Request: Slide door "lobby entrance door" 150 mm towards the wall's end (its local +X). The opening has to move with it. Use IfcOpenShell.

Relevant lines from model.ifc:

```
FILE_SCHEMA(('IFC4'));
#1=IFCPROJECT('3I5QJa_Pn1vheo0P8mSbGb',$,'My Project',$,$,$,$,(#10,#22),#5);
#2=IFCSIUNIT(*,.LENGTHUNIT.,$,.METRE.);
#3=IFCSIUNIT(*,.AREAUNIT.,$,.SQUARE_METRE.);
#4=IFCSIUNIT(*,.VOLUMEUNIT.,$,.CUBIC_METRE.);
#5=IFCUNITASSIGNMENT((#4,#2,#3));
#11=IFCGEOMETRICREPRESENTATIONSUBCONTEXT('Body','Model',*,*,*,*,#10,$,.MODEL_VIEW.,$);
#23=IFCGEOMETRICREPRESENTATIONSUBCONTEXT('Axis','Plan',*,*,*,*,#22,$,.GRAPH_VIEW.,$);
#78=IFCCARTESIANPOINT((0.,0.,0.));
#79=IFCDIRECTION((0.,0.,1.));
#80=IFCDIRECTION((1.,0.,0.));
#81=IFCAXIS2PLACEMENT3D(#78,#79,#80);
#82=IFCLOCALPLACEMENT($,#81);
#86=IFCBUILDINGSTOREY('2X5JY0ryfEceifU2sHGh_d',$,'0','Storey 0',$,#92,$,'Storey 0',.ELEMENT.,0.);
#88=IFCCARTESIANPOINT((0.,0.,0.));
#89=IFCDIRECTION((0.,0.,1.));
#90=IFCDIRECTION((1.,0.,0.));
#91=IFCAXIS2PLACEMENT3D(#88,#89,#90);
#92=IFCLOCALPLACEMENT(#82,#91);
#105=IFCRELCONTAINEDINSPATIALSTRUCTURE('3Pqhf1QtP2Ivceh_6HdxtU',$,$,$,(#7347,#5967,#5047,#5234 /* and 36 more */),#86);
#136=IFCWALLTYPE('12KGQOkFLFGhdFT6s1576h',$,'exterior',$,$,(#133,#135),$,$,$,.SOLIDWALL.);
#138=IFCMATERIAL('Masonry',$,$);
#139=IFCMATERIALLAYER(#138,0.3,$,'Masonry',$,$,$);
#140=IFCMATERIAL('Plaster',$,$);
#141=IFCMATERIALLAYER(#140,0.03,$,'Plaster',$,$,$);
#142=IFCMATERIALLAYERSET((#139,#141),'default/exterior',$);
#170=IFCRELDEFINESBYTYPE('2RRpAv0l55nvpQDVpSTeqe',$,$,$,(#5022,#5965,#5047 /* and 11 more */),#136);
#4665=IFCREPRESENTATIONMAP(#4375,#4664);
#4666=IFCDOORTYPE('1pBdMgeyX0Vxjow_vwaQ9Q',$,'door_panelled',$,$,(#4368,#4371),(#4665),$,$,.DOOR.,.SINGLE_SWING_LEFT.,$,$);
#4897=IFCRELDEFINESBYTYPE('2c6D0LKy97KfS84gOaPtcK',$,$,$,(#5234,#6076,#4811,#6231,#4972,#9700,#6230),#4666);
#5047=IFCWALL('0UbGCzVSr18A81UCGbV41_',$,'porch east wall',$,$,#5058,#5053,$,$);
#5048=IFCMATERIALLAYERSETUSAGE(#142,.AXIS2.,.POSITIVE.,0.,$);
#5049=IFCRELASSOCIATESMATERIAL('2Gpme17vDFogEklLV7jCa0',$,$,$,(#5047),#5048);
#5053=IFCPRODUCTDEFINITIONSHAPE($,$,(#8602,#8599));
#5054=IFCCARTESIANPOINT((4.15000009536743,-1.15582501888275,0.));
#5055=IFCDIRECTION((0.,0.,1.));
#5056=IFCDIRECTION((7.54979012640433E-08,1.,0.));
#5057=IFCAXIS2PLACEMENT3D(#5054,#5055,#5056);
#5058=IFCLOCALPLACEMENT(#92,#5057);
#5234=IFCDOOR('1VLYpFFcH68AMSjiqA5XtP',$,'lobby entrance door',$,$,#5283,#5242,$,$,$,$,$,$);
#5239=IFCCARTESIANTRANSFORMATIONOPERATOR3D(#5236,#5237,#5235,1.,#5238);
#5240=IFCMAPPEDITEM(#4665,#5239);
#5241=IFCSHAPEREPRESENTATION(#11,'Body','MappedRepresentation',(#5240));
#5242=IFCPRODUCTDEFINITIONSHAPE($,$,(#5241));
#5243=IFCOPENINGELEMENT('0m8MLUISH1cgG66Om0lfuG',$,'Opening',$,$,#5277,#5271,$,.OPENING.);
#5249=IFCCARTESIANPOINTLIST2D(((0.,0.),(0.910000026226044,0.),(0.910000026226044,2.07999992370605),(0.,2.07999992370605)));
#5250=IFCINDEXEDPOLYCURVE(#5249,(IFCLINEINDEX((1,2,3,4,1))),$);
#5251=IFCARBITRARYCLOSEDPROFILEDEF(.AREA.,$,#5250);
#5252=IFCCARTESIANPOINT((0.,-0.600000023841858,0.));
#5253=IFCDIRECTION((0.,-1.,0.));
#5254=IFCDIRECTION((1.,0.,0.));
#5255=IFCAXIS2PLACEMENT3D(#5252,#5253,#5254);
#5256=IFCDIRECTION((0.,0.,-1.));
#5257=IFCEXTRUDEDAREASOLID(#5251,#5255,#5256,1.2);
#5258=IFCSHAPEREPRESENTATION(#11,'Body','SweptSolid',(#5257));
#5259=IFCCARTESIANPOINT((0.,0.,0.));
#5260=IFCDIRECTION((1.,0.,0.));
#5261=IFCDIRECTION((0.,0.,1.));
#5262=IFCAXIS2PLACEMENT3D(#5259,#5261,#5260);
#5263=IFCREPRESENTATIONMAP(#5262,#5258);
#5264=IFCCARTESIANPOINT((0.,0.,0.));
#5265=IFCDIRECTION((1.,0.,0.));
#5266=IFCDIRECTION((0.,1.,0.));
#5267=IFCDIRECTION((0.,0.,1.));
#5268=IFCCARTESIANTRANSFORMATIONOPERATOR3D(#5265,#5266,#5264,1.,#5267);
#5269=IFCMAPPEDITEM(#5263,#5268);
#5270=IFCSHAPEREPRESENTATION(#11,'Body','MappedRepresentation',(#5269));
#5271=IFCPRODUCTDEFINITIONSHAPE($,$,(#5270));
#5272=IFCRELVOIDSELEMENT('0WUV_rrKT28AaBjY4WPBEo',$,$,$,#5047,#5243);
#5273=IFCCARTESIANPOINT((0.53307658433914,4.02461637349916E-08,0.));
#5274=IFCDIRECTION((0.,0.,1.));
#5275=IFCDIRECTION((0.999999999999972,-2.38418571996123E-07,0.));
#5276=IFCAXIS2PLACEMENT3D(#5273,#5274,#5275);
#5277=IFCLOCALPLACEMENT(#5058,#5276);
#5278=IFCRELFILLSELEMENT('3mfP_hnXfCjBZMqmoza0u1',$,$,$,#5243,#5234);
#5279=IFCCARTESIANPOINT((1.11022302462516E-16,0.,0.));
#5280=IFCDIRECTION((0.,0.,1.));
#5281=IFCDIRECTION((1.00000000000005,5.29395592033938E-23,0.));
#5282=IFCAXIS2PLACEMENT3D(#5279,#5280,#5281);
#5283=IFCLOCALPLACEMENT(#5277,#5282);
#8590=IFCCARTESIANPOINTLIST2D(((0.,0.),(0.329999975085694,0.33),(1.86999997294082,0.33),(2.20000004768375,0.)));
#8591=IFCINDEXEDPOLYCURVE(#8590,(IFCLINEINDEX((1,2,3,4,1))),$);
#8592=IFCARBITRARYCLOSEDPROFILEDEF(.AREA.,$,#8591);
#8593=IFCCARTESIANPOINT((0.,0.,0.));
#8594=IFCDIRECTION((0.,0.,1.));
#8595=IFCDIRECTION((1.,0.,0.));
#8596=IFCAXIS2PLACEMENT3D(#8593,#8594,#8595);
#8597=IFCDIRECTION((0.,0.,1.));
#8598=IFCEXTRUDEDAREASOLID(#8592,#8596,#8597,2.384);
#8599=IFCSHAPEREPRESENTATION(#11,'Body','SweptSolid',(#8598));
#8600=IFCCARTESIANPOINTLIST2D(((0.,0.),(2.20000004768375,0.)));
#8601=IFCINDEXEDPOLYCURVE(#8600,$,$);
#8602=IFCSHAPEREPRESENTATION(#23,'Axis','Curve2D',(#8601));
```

```python
import ifcopenshell
import ifcopenshell.api.geometry
import ifcopenshell.util.placement
import ifcopenshell.util.unit

model = ifcopenshell.open("model.ifc")
unit_scale = ifcopenshell.util.unit.calculate_unit_scale(model)

door = model.by_guid("1VLYpFFcH68AMSjiqA5XtP")
opening = door.FillsVoids[0].RelatingOpeningElement
wall = opening.VoidsElements[0].RelatingBuildingElement

wall_matrix = ifcopenshell.util.placement.get_local_placement(wall.ObjectPlacement)
shift = wall_matrix[:3, 0] * 0.15 / unit_scale
before = ifcopenshell.util.placement.get_local_placement(door.ObjectPlacement)[:3, 3].copy()

# The door is placed relative to its opening, so it follows when the opening moves.
matrix = ifcopenshell.util.placement.get_local_placement(opening.ObjectPlacement)
matrix[:3, 3] += shift
ifcopenshell.api.geometry.edit_object_placement(
    model, product=opening, matrix=matrix, is_si=False, should_transform_children=True
)

after = ifcopenshell.util.placement.get_local_placement(door.ObjectPlacement)[:3, 3]
print("door moved by", (after - before).round(3) + 0.0)

model.write("model_edited.ifc")
```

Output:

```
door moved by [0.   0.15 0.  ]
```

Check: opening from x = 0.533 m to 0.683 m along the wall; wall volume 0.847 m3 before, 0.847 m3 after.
